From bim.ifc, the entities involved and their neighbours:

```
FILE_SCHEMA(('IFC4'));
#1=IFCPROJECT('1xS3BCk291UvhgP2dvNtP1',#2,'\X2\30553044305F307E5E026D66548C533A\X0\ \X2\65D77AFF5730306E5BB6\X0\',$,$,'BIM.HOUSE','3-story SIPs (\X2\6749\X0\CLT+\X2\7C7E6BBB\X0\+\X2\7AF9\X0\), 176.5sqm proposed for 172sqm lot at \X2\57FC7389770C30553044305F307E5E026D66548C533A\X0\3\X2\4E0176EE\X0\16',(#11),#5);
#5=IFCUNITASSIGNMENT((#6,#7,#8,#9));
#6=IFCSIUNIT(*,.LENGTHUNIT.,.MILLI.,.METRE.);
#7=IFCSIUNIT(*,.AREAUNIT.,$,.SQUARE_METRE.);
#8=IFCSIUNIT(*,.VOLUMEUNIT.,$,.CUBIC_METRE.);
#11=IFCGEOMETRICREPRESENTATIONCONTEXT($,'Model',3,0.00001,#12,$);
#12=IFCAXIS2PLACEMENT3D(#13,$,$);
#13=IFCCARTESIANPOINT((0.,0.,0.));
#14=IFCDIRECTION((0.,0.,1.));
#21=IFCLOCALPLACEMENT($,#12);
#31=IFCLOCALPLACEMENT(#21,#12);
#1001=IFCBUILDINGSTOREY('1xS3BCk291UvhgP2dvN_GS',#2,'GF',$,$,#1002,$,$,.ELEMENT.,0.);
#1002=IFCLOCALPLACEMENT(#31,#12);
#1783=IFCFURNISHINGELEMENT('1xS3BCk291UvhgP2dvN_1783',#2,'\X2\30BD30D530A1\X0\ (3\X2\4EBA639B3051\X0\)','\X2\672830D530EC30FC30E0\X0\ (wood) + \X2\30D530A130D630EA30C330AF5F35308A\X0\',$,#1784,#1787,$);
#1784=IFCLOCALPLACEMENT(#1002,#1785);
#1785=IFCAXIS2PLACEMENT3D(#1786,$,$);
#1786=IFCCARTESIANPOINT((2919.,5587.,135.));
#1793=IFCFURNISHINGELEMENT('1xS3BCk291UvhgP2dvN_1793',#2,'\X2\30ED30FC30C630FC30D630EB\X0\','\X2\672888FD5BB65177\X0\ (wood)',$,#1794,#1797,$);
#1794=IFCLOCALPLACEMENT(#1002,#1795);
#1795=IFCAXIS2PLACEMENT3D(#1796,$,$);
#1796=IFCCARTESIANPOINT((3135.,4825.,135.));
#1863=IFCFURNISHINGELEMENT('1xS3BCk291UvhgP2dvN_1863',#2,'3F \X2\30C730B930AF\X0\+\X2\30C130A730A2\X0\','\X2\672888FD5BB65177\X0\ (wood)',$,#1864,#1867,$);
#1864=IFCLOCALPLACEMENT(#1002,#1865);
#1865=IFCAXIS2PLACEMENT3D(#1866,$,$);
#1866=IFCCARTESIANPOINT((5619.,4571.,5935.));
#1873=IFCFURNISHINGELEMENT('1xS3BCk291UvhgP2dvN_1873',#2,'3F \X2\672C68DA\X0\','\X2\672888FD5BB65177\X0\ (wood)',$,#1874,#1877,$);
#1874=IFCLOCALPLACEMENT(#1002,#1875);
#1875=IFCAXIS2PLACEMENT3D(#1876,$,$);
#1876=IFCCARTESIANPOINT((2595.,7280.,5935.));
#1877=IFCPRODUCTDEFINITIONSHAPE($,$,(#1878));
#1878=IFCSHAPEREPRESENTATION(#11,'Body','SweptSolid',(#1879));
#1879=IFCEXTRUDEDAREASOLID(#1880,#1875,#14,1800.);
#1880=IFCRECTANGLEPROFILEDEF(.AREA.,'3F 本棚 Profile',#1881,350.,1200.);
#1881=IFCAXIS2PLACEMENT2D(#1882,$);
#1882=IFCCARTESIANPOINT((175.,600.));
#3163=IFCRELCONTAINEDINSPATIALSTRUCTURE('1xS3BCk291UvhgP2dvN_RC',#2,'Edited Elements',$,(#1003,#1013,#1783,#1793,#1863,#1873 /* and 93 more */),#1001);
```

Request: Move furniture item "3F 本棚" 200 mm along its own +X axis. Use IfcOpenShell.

```python
import ifcopenshell
import ifcopenshell.api.geometry
import ifcopenshell.util.placement
import ifcopenshell.util.unit

model = ifcopenshell.open("bim.ifc")
unit_scale = ifcopenshell.util.unit.calculate_unit_scale(model)

item = model.by_id(1873)
matrix = ifcopenshell.util.placement.get_local_placement(item.ObjectPlacement)
matrix[:3, 3] += matrix[:3, 0] * 0.2 / unit_scale
ifcopenshell.api.geometry.edit_object_placement(model, product=item, matrix=matrix, is_si=False)

print(ifcopenshell.util.placement.get_local_placement(item.ObjectPlacement).round(3) + 0.0)

model.write("bim_rev.ifc")
```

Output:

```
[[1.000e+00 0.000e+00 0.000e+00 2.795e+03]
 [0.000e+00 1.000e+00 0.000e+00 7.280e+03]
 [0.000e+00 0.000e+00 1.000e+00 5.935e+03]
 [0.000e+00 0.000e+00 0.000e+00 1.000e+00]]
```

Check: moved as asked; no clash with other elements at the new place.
